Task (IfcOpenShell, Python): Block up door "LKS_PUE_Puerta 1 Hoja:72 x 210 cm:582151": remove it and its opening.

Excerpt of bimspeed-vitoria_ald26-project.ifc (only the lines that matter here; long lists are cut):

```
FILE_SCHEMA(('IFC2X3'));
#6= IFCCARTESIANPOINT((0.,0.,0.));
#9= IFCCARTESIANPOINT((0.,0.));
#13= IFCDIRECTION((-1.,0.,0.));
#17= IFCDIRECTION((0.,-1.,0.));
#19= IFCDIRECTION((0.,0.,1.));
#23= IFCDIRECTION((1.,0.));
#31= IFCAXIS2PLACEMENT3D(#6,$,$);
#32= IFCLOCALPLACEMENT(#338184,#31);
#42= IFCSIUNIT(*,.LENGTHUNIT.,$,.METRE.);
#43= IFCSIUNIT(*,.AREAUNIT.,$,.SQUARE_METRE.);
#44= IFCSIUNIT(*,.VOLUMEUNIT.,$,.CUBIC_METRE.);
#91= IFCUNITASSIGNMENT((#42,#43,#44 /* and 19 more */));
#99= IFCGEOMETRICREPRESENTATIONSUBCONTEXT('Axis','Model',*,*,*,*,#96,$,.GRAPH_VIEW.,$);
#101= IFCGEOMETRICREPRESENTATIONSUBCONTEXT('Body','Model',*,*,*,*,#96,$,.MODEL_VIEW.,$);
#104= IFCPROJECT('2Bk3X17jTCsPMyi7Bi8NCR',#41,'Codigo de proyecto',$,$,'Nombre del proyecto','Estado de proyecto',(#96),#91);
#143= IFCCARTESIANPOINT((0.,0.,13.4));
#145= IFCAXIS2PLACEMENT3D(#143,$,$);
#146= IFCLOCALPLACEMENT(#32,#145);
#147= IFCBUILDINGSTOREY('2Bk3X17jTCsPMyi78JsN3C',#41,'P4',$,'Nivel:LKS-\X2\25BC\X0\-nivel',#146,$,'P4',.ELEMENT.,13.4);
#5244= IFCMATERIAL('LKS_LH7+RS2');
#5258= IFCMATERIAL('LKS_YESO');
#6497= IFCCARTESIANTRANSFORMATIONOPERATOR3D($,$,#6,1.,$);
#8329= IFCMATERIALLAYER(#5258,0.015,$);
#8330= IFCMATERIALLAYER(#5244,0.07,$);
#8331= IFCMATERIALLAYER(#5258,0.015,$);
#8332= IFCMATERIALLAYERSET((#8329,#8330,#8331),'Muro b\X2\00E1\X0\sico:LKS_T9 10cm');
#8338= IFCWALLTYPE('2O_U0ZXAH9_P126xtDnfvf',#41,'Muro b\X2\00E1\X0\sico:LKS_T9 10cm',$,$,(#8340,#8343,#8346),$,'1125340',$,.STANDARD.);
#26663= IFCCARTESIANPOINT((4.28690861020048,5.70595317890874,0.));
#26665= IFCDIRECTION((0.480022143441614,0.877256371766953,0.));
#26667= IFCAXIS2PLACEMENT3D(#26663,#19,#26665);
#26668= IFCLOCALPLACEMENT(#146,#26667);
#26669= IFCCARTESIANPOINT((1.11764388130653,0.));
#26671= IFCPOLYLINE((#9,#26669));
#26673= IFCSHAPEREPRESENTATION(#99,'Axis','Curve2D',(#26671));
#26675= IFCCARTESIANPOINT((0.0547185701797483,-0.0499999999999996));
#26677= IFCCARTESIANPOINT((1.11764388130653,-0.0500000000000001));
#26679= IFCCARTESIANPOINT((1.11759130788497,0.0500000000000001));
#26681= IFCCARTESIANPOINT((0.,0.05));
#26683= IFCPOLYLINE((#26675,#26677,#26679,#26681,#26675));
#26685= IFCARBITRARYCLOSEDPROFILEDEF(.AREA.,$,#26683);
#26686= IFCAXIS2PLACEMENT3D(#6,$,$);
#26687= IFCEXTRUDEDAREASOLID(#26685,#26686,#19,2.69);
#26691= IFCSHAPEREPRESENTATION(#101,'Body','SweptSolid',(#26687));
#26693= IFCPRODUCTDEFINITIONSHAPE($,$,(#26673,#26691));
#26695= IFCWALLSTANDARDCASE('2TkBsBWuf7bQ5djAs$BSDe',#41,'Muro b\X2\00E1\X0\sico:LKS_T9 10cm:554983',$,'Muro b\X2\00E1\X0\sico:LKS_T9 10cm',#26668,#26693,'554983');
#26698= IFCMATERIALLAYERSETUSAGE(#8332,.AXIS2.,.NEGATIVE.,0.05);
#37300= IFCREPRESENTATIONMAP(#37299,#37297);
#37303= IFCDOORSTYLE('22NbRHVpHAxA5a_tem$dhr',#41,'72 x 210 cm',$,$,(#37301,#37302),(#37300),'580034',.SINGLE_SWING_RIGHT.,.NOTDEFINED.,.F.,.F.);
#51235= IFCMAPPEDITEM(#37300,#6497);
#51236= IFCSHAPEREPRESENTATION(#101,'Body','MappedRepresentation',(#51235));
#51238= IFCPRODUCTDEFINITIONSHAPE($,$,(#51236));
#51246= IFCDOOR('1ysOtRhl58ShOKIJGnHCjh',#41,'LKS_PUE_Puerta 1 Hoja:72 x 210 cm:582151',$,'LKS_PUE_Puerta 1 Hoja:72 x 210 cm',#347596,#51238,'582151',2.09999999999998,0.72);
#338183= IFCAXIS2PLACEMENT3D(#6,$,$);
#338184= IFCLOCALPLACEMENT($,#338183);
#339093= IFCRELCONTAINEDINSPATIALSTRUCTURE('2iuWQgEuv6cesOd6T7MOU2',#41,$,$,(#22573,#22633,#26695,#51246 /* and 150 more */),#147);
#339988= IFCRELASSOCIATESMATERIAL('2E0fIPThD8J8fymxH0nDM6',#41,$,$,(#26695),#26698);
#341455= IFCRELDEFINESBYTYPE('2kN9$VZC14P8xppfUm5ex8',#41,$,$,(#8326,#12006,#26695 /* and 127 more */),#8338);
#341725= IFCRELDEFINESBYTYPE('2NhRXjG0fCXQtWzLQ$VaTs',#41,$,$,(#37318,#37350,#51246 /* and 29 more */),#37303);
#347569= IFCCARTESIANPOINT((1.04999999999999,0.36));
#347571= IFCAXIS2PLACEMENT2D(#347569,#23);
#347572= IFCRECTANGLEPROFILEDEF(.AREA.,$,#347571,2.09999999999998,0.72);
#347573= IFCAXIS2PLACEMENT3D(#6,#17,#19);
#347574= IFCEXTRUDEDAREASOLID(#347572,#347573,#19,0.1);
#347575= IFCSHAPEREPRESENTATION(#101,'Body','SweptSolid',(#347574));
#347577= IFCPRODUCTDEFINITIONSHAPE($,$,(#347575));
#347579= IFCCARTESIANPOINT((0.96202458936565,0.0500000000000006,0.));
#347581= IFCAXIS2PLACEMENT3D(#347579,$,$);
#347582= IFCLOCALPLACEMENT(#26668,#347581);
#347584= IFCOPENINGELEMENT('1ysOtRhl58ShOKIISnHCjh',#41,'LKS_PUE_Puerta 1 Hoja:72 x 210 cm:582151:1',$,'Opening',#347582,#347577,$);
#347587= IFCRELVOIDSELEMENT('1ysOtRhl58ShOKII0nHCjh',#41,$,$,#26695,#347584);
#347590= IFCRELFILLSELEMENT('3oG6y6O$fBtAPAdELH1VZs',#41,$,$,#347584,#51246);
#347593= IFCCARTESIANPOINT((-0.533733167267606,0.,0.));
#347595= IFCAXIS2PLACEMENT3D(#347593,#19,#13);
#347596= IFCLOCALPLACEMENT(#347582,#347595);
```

```python
import ifcopenshell
import ifcopenshell.api.feature
import ifcopenshell.api.root
import ifcopenshell.geom
import ifcopenshell.util.shape

model = ifcopenshell.open("bimspeed-vitoria_ald26-project.ifc")
settings = ifcopenshell.geom.settings()


def volume(element):
    """Net volume in cubic metres, openings subtracted."""
    shape = ifcopenshell.geom.create_shape(settings, element)
    return ifcopenshell.util.shape.get_volume(shape.geometry)


door = model.by_guid("1ysOtRhl58ShOKIJGnHCjh")
opening = door.FillsVoids[0].RelatingOpeningElement
wall = opening.VoidsElements[0].RelatingBuildingElement
before = volume(wall)

ifcopenshell.api.root.remove_product(model, product=door)
ifcopenshell.api.feature.remove_feature(model, feature=opening)

after = volume(wall)

print(f"wall volume {before:.3f} -> {after:.3f} m3")

model.write("bimspeed-vitoria_ald26-project-out.ifc")
```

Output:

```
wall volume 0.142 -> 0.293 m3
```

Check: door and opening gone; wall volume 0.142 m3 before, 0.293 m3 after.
